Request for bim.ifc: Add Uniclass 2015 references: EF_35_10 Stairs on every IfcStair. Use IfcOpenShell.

First a look at what the model holds.

```python
import ifcopenshell

model = ifcopenshell.open("bim.ifc")
print(model.schema)
print("classifications:", [c.Name for c in model.by_type("IfcClassification")])
for ifc_class in ("IfcDoor", "IfcRoof", "IfcStair", "IfcWall", "IfcWindow"):
    print(ifc_class, len(model.by_type(ifc_class)))
```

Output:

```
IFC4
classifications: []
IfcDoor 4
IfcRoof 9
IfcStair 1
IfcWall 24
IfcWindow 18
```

```python
import ifcopenshell
import ifcopenshell.api.classification

model = ifcopenshell.open("bim.ifc")

system = ifcopenshell.api.classification.add_classification(model, classification="Uniclass 2015")

codes = {
    "IfcStair": ("EF_35_10", "Stairs"),
}
for ifc_class, (code, name) in codes.items():
    products = model.by_type(ifc_class)
    ifcopenshell.api.classification.add_reference(
        model, products=products, classification=system, identification=code, name=name
    )
    print(code, len(products))

model.write("bim_rev.ifc")
```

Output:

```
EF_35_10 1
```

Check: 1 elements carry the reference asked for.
